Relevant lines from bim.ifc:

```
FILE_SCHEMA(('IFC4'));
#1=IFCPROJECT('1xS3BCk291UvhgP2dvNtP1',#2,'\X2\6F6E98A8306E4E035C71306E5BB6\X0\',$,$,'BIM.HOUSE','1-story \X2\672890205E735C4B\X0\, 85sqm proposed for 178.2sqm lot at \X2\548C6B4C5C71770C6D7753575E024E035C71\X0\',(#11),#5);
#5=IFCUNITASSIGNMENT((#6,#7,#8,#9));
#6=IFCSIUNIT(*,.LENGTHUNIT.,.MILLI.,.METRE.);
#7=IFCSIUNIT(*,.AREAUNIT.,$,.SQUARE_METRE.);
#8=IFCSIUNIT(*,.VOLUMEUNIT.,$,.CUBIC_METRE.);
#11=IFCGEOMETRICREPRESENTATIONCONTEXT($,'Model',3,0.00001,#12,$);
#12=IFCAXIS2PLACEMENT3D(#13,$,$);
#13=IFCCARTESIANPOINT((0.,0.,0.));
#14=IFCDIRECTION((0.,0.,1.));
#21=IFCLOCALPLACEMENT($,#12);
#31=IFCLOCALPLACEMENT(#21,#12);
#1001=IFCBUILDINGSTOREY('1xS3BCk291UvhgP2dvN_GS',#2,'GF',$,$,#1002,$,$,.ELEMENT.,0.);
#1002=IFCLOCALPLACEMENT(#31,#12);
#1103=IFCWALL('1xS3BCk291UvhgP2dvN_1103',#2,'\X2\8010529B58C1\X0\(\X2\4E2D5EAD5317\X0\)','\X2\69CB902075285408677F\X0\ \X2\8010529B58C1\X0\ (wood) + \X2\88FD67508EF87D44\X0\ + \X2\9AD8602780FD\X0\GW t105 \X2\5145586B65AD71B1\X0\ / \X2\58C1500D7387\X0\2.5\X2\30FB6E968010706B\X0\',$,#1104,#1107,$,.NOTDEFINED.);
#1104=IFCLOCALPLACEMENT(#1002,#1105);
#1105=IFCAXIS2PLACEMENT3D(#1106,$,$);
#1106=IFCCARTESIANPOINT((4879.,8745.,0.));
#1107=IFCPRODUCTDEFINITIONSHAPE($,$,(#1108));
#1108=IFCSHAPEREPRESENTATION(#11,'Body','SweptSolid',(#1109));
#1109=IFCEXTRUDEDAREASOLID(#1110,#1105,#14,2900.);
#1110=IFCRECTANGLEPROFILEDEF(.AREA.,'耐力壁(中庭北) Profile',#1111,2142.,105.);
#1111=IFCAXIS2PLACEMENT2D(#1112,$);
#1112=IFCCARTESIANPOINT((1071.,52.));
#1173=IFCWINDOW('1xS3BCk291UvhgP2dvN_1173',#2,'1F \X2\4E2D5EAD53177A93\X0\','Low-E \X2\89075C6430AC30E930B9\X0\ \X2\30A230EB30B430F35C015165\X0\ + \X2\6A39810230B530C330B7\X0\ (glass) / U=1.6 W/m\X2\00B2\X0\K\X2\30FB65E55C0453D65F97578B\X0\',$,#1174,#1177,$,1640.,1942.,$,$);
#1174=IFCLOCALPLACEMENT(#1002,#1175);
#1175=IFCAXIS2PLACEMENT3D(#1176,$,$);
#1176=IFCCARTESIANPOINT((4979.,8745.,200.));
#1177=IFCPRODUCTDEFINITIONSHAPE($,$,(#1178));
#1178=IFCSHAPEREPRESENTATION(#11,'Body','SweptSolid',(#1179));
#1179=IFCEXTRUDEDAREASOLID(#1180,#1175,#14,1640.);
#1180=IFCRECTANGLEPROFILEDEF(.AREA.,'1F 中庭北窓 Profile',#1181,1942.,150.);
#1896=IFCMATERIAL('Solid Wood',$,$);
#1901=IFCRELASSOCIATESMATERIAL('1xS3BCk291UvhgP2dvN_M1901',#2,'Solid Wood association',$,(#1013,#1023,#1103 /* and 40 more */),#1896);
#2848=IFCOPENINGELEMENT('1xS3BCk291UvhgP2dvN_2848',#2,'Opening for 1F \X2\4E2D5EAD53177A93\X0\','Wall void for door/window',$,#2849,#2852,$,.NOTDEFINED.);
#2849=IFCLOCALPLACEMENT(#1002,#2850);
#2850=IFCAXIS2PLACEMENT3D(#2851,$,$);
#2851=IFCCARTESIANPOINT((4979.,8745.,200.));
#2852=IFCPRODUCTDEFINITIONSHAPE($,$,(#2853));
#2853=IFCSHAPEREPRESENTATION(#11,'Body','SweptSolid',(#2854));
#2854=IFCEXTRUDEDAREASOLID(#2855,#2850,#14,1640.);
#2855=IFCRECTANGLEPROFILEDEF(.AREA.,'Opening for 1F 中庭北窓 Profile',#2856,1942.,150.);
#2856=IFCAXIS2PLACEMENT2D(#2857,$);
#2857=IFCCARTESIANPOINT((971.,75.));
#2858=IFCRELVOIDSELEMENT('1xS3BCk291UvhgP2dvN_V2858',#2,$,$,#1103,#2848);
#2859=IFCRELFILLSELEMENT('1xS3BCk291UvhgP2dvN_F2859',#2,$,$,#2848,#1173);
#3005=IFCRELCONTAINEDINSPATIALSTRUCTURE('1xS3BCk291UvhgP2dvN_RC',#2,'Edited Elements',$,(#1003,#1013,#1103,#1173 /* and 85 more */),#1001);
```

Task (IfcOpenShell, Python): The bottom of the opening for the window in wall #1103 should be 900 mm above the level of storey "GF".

```python
import numpy as np
import ifcopenshell
import ifcopenshell.api.geometry
import ifcopenshell.geom
import ifcopenshell.util.element
import ifcopenshell.util.placement
import ifcopenshell.util.shape
import ifcopenshell.util.unit

model = ifcopenshell.open("bim.ifc")
unit_scale = ifcopenshell.util.unit.calculate_unit_scale(model)

window = model.by_guid("1xS3BCk291UvhgP2dvN_1173")
opening = window.FillsVoids[0].RelatingOpeningElement
storey = ifcopenshell.util.element.get_container(window, ifc_class="IfcBuildingStorey")
level = ifcopenshell.util.placement.get_local_placement(storey.ObjectPlacement)[2, 3]

# The opening's origin need not be at the sill, so measure its lowest point.
shape = ifcopenshell.geom.create_shape(ifcopenshell.geom.settings(), opening)
bottom = ifcopenshell.util.shape.get_shape_bottom_elevation(shape, shape.geometry) / unit_scale
dz = level + 0.9 / unit_scale - bottom

shift = np.array([0.0, 0.0, dz])
# The window is not placed relative to its opening, so move both.
for product in (opening, window):
    matrix = ifcopenshell.util.placement.get_local_placement(product.ObjectPlacement)
    matrix[:3, 3] += shift
    ifcopenshell.api.geometry.edit_object_placement(model, product=product, matrix=matrix, is_si=False)

print(f"moved by {dz * unit_scale:+.3f} m")

model.write("bim_edited.ifc")
```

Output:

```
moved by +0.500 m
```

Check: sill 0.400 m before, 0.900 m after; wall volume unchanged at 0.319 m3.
